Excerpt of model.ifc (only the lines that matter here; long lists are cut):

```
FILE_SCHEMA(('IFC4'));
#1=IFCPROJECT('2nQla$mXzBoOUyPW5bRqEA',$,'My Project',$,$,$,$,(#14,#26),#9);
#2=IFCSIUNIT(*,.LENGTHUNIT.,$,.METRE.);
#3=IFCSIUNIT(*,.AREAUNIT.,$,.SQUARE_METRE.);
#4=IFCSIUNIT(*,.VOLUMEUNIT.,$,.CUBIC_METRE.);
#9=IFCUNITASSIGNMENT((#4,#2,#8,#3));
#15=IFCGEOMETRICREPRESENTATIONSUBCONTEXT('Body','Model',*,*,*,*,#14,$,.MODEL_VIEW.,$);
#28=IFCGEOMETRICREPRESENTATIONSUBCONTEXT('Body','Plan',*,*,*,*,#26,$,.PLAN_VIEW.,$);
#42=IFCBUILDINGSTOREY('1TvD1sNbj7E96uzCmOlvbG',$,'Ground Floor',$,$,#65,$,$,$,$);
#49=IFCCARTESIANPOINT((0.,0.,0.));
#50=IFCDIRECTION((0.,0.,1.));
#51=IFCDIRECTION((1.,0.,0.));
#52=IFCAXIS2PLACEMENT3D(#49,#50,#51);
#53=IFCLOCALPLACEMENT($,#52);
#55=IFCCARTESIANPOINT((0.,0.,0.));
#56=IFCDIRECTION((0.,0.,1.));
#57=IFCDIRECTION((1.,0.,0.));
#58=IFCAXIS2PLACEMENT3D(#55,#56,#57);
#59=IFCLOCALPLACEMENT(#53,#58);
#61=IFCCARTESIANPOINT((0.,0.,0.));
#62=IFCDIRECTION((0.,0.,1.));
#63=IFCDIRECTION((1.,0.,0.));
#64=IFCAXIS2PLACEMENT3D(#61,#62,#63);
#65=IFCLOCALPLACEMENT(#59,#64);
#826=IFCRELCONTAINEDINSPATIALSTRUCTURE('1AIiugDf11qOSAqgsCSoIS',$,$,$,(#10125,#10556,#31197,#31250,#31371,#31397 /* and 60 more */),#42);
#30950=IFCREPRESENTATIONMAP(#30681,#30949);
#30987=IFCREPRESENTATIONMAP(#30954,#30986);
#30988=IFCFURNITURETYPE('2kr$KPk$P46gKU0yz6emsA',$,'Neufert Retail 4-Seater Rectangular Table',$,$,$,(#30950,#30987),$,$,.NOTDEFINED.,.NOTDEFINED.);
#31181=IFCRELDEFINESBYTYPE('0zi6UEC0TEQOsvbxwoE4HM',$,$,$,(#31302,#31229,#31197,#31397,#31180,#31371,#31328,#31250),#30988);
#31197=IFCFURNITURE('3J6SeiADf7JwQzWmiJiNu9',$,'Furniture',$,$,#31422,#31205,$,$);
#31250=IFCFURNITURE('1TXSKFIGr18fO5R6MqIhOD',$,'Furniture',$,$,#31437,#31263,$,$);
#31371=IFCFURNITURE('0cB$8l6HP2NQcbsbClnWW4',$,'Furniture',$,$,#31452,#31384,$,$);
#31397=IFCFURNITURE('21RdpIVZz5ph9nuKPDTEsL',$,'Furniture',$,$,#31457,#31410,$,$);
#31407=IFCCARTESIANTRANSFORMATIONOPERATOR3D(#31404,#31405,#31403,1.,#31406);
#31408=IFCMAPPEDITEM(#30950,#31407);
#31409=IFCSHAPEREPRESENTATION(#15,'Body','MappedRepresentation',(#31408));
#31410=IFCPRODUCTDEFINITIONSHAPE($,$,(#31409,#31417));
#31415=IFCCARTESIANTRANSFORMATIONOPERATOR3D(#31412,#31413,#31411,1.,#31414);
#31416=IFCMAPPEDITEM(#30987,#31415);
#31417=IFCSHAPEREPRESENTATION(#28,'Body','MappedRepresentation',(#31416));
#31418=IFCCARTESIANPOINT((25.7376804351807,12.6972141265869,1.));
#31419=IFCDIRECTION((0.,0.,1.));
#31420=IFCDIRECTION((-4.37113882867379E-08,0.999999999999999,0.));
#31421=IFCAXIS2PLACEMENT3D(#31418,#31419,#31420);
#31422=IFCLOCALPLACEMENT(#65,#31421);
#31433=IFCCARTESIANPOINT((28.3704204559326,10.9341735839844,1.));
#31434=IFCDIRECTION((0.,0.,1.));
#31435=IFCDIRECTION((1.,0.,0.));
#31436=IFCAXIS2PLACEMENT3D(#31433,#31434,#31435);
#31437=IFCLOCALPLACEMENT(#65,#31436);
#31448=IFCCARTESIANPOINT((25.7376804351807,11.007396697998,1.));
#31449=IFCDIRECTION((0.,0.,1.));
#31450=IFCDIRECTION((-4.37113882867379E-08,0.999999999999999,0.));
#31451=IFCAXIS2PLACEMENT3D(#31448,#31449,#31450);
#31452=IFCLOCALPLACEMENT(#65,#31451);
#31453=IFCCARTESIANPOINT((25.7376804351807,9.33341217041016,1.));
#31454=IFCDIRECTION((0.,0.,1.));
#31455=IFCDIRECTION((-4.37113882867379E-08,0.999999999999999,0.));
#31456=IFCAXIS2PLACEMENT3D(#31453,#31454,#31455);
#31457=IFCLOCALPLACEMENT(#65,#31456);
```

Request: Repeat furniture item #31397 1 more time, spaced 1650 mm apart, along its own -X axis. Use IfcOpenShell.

```python
import ifcopenshell
import ifcopenshell.api.geometry
import ifcopenshell.api.root
import ifcopenshell.util.element
import ifcopenshell.util.placement
import ifcopenshell.util.unit

model = ifcopenshell.open("model.ifc")
unit_scale = ifcopenshell.util.unit.calculate_unit_scale(model)

source = model.by_id(31397)
base = ifcopenshell.util.placement.get_local_placement(source.ObjectPlacement)
step = -base[:3, 0] * 1.65 / unit_scale

for i in range(1, 2):
    copy = ifcopenshell.api.root.copy_class(model, product=source)
    copy.Representation = ifcopenshell.util.element.copy_deep(
        model, source.Representation, exclude=["IfcGeometricRepresentationContext", "IfcRepresentationMap"]
    )
    matrix = base.copy()
    matrix[:3, 3] += i * step
    print("added at", matrix[:3, 3].round(3) + 0.0)
    ifcopenshell.api.geometry.edit_object_placement(model, product=copy, matrix=matrix, is_si=False)

model.write("model_rev.ifc")
```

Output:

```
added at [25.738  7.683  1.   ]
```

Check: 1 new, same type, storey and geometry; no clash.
